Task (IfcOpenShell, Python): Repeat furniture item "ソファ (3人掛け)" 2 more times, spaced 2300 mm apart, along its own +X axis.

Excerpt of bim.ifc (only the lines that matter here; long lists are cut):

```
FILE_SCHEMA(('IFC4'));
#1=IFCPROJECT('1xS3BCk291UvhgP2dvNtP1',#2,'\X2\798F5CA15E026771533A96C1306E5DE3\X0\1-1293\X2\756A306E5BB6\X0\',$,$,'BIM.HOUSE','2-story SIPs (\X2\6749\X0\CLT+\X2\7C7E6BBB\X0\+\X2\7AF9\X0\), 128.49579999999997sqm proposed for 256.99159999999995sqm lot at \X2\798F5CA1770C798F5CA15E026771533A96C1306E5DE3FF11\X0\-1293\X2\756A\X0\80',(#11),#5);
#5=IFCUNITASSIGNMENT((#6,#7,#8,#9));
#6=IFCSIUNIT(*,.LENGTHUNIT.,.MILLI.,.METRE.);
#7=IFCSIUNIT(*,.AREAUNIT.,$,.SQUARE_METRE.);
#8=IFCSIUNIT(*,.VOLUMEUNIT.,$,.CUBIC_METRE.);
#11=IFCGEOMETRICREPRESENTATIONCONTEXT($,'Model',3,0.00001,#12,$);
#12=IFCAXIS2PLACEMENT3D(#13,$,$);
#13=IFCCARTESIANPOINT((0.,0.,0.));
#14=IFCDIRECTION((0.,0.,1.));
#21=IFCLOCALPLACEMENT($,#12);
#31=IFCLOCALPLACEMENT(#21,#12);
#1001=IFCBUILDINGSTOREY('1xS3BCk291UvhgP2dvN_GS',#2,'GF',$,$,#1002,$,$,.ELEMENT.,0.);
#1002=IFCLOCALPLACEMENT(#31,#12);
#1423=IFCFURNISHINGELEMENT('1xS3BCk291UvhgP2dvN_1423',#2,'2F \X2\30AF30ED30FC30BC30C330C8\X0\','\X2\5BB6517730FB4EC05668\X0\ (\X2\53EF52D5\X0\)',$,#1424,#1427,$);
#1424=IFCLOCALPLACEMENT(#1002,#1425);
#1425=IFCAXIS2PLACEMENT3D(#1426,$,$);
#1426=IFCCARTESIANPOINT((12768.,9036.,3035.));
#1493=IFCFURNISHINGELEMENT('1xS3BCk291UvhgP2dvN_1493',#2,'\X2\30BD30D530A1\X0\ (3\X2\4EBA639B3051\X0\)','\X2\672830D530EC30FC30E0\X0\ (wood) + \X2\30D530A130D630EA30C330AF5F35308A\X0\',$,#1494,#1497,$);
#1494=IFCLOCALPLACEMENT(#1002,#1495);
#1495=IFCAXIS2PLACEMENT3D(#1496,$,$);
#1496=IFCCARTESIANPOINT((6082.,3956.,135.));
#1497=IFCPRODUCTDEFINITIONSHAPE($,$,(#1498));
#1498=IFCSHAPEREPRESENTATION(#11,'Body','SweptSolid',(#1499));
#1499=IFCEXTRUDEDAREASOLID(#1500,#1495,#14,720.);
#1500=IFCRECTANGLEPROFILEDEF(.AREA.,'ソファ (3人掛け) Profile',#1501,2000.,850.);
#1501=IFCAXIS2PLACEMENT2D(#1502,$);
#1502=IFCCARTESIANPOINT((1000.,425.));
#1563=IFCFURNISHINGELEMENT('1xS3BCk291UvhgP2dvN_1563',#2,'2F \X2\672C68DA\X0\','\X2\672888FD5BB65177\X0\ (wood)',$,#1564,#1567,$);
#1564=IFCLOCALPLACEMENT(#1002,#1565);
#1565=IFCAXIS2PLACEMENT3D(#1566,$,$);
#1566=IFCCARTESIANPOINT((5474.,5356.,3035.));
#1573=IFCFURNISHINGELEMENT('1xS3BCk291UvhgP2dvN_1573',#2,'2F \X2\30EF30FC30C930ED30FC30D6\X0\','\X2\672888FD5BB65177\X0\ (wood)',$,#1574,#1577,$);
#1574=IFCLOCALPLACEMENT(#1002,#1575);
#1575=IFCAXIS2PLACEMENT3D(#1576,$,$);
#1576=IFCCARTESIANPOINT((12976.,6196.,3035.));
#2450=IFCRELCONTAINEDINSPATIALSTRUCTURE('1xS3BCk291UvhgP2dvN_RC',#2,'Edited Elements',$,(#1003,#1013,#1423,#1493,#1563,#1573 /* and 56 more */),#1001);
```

```python
import ifcopenshell
import ifcopenshell.api.geometry
import ifcopenshell.api.root
import ifcopenshell.util.element
import ifcopenshell.util.placement
import ifcopenshell.util.unit

model = ifcopenshell.open("bim.ifc")
unit_scale = ifcopenshell.util.unit.calculate_unit_scale(model)


def reuse_history(source, copy):
    """copy_class also copies each property set's owner history, people and application; keep the originals."""
    for rel in copy.IsDefinedBy:
        if rel.is_a("IfcRelDefinesByProperties") and (history := rel.RelatingPropertyDefinition.OwnerHistory):
            rel.RelatingPropertyDefinition.OwnerHistory = source.OwnerHistory
            ifcopenshell.util.element.remove_deep2(model, history)


source = model.by_id(1493)
base = ifcopenshell.util.placement.get_local_placement(source.ObjectPlacement)
step = base[:3, 0] * 2.3 / unit_scale

for i in range(1, 3):
    copy = ifcopenshell.api.root.copy_class(model, product=source)
    copy.Representation = ifcopenshell.util.element.copy_deep(
        model, source.Representation, exclude=["IfcGeometricRepresentationContext", "IfcRepresentationMap"]
    )
    reuse_history(source, copy)
    matrix = base.copy()
    matrix[:3, 3] += i * step
    print("added at", matrix[:3, 3].round(3) + 0.0)
    ifcopenshell.api.geometry.edit_object_placement(model, product=copy, matrix=matrix, is_si=False)

model.write("bim-out.ifc")
```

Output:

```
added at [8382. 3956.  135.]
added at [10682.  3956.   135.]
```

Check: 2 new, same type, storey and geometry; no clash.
